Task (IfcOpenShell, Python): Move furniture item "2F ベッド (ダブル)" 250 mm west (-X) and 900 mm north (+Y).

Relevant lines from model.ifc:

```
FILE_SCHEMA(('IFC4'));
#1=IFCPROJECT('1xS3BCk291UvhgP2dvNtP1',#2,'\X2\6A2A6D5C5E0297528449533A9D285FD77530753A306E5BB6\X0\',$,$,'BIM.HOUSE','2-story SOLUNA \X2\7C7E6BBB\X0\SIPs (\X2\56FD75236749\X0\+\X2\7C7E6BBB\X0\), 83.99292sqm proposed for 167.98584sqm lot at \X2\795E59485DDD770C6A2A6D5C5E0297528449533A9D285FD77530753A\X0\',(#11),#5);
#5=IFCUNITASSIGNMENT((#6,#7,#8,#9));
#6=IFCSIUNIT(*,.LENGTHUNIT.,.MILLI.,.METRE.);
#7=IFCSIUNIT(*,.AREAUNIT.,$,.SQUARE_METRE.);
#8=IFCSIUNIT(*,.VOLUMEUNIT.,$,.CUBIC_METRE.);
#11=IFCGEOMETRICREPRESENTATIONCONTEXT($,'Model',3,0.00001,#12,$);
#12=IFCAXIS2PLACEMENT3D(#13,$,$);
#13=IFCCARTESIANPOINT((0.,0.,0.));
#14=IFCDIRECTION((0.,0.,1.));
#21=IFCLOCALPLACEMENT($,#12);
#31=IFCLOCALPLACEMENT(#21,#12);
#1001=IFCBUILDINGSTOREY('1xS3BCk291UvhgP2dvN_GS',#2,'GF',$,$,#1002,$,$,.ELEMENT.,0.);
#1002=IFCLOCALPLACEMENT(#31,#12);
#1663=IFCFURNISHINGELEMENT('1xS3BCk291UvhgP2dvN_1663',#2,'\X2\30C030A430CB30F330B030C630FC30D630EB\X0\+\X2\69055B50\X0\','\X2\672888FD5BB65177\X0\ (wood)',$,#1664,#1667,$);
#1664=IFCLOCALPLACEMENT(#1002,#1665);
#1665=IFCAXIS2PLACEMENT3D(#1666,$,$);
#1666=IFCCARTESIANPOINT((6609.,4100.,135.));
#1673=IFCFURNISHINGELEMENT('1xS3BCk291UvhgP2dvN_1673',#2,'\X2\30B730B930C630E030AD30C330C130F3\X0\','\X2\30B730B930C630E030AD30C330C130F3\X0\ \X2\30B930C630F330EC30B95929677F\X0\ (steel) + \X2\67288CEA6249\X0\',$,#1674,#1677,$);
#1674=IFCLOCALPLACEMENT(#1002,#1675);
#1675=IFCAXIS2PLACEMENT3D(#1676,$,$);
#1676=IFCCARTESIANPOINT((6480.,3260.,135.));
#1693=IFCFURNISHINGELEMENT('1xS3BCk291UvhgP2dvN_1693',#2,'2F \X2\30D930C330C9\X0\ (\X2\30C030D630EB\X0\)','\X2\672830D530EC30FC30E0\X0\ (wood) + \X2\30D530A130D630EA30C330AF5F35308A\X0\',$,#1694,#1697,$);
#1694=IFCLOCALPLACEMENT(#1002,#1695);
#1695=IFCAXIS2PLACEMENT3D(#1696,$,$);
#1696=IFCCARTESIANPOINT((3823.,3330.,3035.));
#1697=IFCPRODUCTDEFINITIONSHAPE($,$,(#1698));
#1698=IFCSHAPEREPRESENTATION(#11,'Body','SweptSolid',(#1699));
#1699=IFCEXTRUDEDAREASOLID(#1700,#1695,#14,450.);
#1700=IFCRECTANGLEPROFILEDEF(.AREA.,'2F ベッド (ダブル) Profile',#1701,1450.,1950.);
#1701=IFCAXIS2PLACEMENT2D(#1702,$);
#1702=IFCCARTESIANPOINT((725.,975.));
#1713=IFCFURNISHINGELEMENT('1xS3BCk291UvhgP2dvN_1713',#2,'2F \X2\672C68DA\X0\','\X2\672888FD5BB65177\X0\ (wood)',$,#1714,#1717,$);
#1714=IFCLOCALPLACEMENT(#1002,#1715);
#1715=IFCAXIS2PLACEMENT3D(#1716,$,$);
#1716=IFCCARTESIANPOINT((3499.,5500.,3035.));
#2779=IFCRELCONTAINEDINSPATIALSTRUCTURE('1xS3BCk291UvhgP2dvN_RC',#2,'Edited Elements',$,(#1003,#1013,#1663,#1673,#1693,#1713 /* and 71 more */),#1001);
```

```python
import ifcopenshell
import ifcopenshell.api.geometry
import ifcopenshell.util.placement

model = ifcopenshell.open("model.ifc")

item = model.by_id(1693)
matrix = ifcopenshell.util.placement.get_local_placement(item.ObjectPlacement)
matrix[0, 3] -= 250.0
matrix[1, 3] += 900.0
ifcopenshell.api.geometry.edit_object_placement(model, product=item, matrix=matrix, is_si=False)

print(ifcopenshell.util.placement.get_local_placement(item.ObjectPlacement).round(3) + 0.0)

model.write("model_updated.ifc")
```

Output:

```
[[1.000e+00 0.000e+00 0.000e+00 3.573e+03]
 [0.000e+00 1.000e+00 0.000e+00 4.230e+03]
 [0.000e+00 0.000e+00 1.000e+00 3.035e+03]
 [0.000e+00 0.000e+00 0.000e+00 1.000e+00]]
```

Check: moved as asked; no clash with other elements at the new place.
